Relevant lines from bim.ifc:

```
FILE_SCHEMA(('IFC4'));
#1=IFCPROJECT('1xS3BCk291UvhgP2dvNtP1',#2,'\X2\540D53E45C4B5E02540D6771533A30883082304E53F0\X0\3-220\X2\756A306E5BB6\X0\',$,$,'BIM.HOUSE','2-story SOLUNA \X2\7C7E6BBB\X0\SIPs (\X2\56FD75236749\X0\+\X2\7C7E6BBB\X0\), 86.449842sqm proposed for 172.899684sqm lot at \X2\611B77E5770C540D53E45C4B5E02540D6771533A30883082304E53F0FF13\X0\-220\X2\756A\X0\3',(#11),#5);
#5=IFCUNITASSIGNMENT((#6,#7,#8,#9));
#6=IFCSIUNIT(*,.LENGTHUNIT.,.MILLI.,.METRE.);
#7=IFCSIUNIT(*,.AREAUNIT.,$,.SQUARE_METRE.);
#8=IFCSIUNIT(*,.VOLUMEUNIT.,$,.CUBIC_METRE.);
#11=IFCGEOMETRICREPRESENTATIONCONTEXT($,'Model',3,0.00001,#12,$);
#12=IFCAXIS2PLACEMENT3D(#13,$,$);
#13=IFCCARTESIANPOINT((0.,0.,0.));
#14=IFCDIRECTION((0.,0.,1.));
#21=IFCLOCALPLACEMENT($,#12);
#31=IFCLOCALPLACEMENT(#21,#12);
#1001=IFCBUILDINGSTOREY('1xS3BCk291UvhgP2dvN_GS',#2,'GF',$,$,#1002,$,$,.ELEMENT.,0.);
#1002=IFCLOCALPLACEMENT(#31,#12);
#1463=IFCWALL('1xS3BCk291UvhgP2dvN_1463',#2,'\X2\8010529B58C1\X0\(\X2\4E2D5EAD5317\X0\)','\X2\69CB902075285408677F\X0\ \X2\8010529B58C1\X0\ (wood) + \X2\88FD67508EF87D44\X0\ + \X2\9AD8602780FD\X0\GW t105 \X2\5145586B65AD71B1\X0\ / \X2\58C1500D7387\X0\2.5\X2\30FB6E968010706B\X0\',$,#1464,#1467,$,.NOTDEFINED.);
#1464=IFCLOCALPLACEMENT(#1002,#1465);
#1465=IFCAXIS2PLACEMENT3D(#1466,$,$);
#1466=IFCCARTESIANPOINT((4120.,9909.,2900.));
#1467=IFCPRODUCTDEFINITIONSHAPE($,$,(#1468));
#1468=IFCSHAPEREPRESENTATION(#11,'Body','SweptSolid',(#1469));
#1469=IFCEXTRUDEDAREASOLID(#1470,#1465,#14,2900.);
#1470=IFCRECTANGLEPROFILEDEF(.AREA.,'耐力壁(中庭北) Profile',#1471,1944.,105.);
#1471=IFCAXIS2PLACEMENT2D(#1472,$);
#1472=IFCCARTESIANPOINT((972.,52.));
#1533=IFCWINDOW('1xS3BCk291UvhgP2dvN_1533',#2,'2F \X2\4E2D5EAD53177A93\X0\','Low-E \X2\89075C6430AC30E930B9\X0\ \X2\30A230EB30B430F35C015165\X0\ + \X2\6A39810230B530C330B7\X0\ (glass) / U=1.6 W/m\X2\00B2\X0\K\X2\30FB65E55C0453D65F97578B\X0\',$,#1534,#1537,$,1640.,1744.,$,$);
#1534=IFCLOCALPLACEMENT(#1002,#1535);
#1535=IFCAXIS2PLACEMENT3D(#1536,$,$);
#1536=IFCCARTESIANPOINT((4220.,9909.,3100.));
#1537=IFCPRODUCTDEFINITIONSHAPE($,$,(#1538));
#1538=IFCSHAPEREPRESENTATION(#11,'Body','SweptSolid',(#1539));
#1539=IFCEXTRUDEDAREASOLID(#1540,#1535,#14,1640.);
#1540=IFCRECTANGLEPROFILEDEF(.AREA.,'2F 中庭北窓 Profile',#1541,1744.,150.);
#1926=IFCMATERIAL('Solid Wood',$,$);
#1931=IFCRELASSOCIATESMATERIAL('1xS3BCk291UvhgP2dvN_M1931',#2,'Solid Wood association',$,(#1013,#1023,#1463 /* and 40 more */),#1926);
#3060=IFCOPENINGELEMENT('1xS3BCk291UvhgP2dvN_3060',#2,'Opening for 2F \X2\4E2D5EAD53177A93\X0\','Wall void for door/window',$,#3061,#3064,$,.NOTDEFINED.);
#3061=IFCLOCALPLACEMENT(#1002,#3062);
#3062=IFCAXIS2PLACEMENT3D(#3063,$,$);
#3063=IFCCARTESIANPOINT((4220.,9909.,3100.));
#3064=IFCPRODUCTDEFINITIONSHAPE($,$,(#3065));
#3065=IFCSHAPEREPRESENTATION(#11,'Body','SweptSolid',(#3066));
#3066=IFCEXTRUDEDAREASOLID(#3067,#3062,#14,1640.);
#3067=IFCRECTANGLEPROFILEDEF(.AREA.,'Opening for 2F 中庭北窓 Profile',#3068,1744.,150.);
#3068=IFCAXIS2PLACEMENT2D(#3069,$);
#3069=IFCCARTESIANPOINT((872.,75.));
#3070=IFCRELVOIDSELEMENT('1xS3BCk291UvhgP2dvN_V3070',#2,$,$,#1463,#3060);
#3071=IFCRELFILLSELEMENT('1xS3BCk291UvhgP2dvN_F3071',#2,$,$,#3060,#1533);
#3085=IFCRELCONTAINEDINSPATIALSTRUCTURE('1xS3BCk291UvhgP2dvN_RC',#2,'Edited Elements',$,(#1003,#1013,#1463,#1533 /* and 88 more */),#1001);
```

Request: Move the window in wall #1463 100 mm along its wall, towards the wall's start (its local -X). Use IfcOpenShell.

```python
import ifcopenshell
import ifcopenshell.api.geometry
import ifcopenshell.util.placement

model = ifcopenshell.open("bim.ifc")

window = model.by_guid("1xS3BCk291UvhgP2dvN_1533")
opening = window.FillsVoids[0].RelatingOpeningElement
wall = opening.VoidsElements[0].RelatingBuildingElement

wall_matrix = ifcopenshell.util.placement.get_local_placement(wall.ObjectPlacement)
shift = wall_matrix[:3, 0] * -100.0
before = ifcopenshell.util.placement.get_local_placement(window.ObjectPlacement)[:3, 3].copy()

# The window is not placed relative to its opening, so move both.
for product in (opening, window):
    matrix = ifcopenshell.util.placement.get_local_placement(product.ObjectPlacement)
    matrix[:3, 3] += shift
    ifcopenshell.api.geometry.edit_object_placement(model, product=product, matrix=matrix, is_si=False)

after = ifcopenshell.util.placement.get_local_placement(window.ObjectPlacement)[:3, 3]
print("window moved by", (after - before).round(3) + 0.0)

model.write("bim_edited.ifc")
```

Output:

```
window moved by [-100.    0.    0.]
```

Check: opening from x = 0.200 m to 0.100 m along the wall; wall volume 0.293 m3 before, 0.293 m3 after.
